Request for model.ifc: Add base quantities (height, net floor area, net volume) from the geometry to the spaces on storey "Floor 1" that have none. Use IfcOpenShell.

First a look at what the model holds.

```python
import ifcopenshell
import ifcopenshell.util.element
import ifcopenshell.util.unit

model = ifcopenshell.open("model.ifc")
print(model.schema)
for unit_type in ("LENGTHUNIT", "AREAUNIT", "VOLUMEUNIT"):
    print(unit_type, ifcopenshell.util.unit.calculate_unit_scale(model, unit_type))
storey = next(s for s in model.by_type("IfcBuildingStorey") if s.Name == "Floor 1")
spaces = [e for e in ifcopenshell.util.element.get_decomposition(storey) if e.is_a("IfcSpace")]
for e in sorted(spaces, key=lambda e: e.id()):
    print(e.id(), e.is_a(), e.Name, list(ifcopenshell.util.element.get_psets(e, qtos_only=True)), sep=" | ")
```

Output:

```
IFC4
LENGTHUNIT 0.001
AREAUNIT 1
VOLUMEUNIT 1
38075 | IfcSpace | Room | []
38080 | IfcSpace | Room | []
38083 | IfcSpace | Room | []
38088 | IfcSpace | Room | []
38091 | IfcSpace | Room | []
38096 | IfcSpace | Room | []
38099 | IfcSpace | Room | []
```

```python
import ifcopenshell
import ifcopenshell.api.pset
import ifcopenshell.geom
import ifcopenshell.util.element
import ifcopenshell.util.shape
import ifcopenshell.util.unit

model = ifcopenshell.open("model.ifc")
unit_scale = ifcopenshell.util.unit.calculate_unit_scale(model)
area_scale = ifcopenshell.util.unit.calculate_unit_scale(model, "AREAUNIT")
volume_scale = ifcopenshell.util.unit.calculate_unit_scale(model, "VOLUMEUNIT")
settings = ifcopenshell.geom.settings()

storey = next(s for s in model.by_type("IfcBuildingStorey") if s.Name == "Floor 1")
spaces = [e for e in ifcopenshell.util.element.get_decomposition(storey) if e.is_a("IfcSpace")]

for e in sorted(spaces, key=lambda e: e.id()):
    if ifcopenshell.util.element.get_psets(e, qtos_only=True, should_inherit=False):
        continue
    # Geometry comes back in metres, in the element's own axes.
    shape = ifcopenshell.geom.create_shape(settings, e)
    values = {
        "Height": ifcopenshell.util.shape.get_z(shape.geometry) / unit_scale,
        "NetFloorArea": ifcopenshell.util.shape.get_footprint_area(shape.geometry) / area_scale,
        "NetVolume": ifcopenshell.util.shape.get_volume(shape.geometry) / volume_scale,
    }
    qto = ifcopenshell.api.pset.add_qto(model, product=e, name="Qto_SpaceBaseQuantities")
    ifcopenshell.api.pset.edit_qto(model, qto=qto, properties=values)
    print(e.id(), {k: round(v, 3) for k, v in values.items()})

model.write("model_rev.ifc")
```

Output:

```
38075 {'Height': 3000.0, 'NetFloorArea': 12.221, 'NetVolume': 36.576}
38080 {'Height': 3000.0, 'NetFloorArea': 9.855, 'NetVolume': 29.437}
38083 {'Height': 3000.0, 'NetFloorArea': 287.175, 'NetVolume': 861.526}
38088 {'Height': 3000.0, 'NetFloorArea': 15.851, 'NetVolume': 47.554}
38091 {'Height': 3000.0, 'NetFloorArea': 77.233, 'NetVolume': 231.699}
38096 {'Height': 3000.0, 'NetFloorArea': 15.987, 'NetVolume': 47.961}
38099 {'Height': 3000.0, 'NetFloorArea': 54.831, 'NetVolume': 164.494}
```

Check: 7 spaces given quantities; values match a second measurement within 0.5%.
